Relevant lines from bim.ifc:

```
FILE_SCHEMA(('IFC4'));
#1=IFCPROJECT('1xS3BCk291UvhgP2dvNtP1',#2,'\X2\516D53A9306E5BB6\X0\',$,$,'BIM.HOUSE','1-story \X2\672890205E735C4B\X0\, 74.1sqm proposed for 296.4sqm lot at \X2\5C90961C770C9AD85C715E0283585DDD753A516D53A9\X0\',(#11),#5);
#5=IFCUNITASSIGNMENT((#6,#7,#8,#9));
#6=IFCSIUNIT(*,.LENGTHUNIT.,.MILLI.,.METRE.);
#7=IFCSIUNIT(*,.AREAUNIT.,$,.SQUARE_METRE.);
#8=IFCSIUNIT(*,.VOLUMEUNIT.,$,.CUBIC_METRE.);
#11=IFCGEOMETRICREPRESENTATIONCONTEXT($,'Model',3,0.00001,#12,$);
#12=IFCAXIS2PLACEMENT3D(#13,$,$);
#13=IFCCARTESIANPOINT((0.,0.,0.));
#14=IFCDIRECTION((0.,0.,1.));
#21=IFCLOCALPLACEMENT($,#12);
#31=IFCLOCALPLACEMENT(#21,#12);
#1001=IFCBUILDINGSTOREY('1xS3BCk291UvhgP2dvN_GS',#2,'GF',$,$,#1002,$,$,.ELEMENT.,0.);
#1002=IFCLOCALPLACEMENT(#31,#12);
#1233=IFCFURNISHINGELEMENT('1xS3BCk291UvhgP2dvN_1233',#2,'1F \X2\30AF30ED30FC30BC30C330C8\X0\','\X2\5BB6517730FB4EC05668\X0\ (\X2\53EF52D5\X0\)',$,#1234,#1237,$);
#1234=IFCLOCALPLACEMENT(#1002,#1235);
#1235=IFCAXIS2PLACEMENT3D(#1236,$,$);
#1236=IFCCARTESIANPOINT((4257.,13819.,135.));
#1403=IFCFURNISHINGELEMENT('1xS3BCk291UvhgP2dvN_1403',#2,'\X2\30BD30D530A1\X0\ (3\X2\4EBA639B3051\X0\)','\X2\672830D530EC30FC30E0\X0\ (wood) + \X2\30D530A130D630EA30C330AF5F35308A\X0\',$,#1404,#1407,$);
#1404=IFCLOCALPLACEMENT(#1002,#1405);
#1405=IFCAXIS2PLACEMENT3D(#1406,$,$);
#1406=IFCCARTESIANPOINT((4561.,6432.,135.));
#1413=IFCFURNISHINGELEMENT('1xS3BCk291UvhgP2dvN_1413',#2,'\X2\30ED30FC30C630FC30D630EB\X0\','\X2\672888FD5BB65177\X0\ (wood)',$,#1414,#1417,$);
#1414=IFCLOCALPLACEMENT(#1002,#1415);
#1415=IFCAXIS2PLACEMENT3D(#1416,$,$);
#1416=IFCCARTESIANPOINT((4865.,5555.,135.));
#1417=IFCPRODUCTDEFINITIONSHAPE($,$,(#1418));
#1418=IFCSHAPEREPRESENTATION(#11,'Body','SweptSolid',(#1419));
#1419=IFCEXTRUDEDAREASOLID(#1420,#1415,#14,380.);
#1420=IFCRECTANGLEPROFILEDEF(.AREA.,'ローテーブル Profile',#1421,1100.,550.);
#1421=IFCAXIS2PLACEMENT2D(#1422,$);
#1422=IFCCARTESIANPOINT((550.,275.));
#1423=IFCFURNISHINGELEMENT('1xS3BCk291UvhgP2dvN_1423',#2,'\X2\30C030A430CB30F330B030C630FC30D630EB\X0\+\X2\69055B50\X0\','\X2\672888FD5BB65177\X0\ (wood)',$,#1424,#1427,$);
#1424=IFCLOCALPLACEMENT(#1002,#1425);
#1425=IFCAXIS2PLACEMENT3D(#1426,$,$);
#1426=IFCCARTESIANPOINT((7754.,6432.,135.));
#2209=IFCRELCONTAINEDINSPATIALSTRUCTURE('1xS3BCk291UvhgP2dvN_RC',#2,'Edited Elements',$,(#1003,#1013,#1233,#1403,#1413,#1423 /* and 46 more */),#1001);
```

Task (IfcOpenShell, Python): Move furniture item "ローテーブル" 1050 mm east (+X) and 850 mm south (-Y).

```python
import ifcopenshell
import ifcopenshell.api.geometry
import ifcopenshell.util.placement
import ifcopenshell.util.unit

model = ifcopenshell.open("bim.ifc")
unit_scale = ifcopenshell.util.unit.calculate_unit_scale(model)

item = model.by_guid("1xS3BCk291UvhgP2dvN_1413")
matrix = ifcopenshell.util.placement.get_local_placement(item.ObjectPlacement)
matrix[0, 3] += 1.05 / unit_scale
matrix[1, 3] -= 0.85 / unit_scale
ifcopenshell.api.geometry.edit_object_placement(model, product=item, matrix=matrix, is_si=False)

print(ifcopenshell.util.placement.get_local_placement(item.ObjectPlacement).round(3) + 0.0)

model.write("bim-out.ifc")
```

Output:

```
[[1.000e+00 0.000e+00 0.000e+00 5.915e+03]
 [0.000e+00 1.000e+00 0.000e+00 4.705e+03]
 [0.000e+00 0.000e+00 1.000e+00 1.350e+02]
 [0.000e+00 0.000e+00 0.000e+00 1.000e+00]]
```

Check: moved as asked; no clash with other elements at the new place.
